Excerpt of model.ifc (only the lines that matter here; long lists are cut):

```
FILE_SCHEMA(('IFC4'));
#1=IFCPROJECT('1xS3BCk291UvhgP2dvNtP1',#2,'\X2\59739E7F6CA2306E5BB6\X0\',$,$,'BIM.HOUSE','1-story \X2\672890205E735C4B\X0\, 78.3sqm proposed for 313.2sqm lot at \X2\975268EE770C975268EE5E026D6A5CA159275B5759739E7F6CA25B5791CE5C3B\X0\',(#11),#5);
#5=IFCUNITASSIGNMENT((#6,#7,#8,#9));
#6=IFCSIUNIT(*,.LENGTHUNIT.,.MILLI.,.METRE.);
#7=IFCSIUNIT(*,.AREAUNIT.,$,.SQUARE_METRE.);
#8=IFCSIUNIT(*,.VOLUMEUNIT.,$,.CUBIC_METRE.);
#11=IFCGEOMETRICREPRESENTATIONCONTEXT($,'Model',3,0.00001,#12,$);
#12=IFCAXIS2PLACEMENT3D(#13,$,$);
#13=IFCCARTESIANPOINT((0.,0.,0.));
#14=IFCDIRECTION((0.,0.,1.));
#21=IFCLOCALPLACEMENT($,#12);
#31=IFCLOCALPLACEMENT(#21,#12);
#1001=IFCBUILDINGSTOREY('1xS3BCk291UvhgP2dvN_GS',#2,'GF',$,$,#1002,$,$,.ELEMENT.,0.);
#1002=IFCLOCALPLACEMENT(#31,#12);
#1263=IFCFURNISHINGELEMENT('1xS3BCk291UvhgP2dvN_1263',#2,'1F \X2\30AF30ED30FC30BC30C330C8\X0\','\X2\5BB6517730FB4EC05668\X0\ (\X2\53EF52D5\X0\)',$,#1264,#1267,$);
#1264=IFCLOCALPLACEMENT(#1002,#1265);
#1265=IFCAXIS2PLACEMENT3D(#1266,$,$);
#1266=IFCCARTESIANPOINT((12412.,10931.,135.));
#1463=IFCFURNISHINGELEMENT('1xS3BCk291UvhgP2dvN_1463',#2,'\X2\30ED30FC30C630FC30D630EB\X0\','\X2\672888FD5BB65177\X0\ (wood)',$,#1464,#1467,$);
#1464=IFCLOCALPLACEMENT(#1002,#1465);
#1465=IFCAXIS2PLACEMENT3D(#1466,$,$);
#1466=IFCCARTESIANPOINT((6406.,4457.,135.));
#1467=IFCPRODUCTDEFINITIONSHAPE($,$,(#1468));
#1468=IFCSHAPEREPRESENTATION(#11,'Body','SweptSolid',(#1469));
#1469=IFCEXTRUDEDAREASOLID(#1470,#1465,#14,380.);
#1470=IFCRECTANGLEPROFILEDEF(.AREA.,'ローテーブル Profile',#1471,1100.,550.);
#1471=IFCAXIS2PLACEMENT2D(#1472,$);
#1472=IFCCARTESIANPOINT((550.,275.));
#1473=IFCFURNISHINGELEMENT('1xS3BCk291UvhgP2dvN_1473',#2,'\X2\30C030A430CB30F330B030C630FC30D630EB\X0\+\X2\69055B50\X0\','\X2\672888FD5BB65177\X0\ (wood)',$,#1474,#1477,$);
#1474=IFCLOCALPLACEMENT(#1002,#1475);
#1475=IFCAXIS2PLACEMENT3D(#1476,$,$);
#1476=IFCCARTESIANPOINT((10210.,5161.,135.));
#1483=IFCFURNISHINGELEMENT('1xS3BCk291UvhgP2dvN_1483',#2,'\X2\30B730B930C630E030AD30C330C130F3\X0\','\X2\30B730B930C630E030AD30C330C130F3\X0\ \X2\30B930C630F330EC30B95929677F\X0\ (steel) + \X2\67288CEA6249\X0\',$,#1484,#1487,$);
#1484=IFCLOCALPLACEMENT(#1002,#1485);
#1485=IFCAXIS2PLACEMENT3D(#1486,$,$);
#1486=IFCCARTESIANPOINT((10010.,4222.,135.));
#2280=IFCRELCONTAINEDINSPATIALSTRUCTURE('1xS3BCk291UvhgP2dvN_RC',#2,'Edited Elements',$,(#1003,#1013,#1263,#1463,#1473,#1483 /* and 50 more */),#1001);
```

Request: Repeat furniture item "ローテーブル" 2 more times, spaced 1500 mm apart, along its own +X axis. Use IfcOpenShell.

```python
import ifcopenshell
import ifcopenshell.api.geometry
import ifcopenshell.api.root
import ifcopenshell.util.element
import ifcopenshell.util.placement
import ifcopenshell.util.unit

model = ifcopenshell.open("model.ifc")
unit_scale = ifcopenshell.util.unit.calculate_unit_scale(model)


def reuse_history(source, copy):
    """copy_class also copies each property set's owner history, people and application; keep the originals."""
    for rel in copy.IsDefinedBy:
        if rel.is_a("IfcRelDefinesByProperties") and (history := rel.RelatingPropertyDefinition.OwnerHistory):
            rel.RelatingPropertyDefinition.OwnerHistory = source.OwnerHistory
            ifcopenshell.util.element.remove_deep2(model, history)


source = model.by_guid("1xS3BCk291UvhgP2dvN_1463")
base = ifcopenshell.util.placement.get_local_placement(source.ObjectPlacement)
step = base[:3, 0] * 1.5 / unit_scale

for i in range(1, 3):
    copy = ifcopenshell.api.root.copy_class(model, product=source)
    copy.Representation = ifcopenshell.util.element.copy_deep(
        model, source.Representation, exclude=["IfcGeometricRepresentationContext", "IfcRepresentationMap"]
    )
    reuse_history(source, copy)
    matrix = base.copy()
    matrix[:3, 3] += i * step
    print("added at", matrix[:3, 3].round(3) + 0.0)
    ifcopenshell.api.geometry.edit_object_placement(model, product=copy, matrix=matrix, is_si=False)

model.write("model_v2.ifc")
```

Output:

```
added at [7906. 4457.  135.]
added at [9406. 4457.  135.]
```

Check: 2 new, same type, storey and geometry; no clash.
